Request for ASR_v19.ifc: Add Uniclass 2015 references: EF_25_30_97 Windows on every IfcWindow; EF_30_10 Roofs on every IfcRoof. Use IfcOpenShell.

First a look at what the model holds.

```python
import ifcopenshell

model = ifcopenshell.open("ASR_v19.ifc")
print(model.schema)
print("classifications:", [c.Name for c in model.by_type("IfcClassification")])
for ifc_class in ("IfcDoor", "IfcRoof", "IfcStair", "IfcWall", "IfcWindow"):
    print(ifc_class, len(model.by_type(ifc_class)))
```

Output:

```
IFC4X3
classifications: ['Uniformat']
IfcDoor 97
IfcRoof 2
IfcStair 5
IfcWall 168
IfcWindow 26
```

```python
import ifcopenshell
import ifcopenshell.api.classification

model = ifcopenshell.open("ASR_v19.ifc")

system = ifcopenshell.api.classification.add_classification(model, classification="Uniclass 2015")

codes = {
    "IfcWindow": ("EF_25_30_97", "Windows"),
    "IfcRoof": ("EF_30_10", "Roofs"),
}
for ifc_class, (code, name) in codes.items():
    products = model.by_type(ifc_class)
    ifcopenshell.api.classification.add_reference(
        model, products=products, classification=system, identification=code, name=name
    )
    print(code, len(products))

model.write("ASR_v19-out.ifc")
```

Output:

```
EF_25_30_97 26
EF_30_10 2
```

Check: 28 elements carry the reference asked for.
